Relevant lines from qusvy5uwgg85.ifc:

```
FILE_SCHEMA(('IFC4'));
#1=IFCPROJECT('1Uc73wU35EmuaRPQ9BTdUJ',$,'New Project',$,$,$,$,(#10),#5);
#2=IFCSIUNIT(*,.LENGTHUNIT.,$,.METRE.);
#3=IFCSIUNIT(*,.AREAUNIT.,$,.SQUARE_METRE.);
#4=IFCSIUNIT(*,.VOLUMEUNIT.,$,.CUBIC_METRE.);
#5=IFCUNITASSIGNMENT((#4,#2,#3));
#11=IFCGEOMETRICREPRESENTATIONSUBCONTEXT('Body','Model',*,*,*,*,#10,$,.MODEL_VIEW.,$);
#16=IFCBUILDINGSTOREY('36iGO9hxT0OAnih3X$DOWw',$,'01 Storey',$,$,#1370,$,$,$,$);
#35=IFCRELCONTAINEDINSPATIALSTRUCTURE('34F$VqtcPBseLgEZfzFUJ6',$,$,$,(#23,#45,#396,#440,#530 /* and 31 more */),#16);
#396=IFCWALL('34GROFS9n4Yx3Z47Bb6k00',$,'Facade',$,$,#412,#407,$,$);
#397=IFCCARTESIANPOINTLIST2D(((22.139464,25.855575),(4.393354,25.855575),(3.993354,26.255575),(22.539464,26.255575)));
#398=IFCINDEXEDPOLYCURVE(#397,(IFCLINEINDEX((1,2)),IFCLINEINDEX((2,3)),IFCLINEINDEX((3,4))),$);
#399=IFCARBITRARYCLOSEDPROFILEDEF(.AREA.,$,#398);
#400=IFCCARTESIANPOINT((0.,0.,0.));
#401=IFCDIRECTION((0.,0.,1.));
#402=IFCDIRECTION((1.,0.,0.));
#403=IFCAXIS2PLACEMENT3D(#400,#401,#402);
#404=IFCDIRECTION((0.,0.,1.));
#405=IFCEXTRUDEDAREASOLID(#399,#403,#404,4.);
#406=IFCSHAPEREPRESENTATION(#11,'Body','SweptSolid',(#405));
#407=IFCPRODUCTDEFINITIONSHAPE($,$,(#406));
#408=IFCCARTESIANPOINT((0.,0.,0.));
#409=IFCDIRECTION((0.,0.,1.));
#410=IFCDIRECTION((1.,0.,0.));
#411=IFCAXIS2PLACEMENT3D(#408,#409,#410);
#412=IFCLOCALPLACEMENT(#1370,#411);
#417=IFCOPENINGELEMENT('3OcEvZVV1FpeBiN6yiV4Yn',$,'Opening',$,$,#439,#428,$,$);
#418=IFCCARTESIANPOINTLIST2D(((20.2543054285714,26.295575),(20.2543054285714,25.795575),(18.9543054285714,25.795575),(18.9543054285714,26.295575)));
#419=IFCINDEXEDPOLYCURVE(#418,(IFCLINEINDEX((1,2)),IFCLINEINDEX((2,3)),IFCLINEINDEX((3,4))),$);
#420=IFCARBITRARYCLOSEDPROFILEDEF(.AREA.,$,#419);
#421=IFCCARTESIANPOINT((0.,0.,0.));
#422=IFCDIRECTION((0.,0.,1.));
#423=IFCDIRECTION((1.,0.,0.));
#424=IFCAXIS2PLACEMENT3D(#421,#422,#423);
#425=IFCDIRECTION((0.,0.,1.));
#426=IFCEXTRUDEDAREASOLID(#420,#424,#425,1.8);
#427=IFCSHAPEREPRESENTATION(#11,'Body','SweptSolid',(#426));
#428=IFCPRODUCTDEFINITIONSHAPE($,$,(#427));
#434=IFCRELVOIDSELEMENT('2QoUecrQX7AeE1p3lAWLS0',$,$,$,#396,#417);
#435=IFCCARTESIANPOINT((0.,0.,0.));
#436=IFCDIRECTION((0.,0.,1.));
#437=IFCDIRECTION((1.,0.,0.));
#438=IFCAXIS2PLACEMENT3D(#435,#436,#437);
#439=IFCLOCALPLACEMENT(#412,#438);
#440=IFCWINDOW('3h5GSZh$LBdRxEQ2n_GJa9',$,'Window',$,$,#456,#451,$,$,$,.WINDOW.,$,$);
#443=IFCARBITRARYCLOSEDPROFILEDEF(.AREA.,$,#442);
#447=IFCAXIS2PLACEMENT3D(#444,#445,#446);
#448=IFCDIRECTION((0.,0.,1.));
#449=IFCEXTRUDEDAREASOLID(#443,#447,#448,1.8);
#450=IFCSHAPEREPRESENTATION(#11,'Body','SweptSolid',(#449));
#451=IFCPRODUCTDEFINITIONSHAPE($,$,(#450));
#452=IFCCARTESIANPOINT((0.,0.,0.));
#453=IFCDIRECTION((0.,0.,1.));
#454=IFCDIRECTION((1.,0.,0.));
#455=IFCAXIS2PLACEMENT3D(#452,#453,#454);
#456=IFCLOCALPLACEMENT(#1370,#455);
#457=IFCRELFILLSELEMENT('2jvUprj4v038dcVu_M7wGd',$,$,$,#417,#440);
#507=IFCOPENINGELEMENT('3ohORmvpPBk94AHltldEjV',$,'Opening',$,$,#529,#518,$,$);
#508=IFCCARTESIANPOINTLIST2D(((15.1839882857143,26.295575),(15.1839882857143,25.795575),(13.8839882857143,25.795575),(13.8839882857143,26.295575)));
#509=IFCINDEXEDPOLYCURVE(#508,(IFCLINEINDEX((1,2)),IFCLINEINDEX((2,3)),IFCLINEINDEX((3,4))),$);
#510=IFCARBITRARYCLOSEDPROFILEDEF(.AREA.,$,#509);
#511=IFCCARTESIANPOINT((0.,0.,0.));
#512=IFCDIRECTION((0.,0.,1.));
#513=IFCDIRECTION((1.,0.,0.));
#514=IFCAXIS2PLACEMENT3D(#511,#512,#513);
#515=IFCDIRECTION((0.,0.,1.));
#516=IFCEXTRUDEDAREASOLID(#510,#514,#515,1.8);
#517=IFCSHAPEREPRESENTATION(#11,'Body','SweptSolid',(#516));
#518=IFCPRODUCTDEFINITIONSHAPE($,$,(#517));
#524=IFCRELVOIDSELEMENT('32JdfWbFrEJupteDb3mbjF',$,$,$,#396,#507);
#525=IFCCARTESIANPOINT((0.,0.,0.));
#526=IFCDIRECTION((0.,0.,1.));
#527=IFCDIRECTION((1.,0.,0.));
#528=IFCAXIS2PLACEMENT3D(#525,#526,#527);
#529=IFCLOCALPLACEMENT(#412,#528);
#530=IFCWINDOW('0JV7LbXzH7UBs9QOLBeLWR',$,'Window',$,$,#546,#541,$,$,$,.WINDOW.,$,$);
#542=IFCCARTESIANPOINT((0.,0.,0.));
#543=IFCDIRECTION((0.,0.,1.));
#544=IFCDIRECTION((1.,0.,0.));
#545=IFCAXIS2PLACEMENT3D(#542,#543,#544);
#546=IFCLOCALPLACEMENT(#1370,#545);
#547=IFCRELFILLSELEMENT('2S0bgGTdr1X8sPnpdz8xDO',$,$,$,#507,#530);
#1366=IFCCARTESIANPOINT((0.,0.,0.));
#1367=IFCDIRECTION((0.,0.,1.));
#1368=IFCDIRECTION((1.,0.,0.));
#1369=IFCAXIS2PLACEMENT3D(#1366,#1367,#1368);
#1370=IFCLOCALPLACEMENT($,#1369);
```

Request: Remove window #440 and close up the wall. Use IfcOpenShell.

```python
import ifcopenshell
import ifcopenshell.api.feature
import ifcopenshell.api.root
import ifcopenshell.geom
import ifcopenshell.util.shape

model = ifcopenshell.open("qusvy5uwgg85.ifc")
settings = ifcopenshell.geom.settings()


def volume(element):
    """Net volume in cubic metres, openings subtracted."""
    shape = ifcopenshell.geom.create_shape(settings, element)
    return ifcopenshell.util.shape.get_volume(shape.geometry)


window = model.by_id(440)
opening = window.FillsVoids[0].RelatingOpeningElement
wall = opening.VoidsElements[0].RelatingBuildingElement
before = volume(wall)

ifcopenshell.api.root.remove_product(model, product=window)
ifcopenshell.api.feature.remove_feature(model, feature=opening)

after = volume(wall)

print(f"wall volume {before:.3f} -> {after:.3f} m3")

model.write("qusvy5uwgg85_updated.ifc")
```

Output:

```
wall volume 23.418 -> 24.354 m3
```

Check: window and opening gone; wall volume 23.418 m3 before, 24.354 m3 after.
